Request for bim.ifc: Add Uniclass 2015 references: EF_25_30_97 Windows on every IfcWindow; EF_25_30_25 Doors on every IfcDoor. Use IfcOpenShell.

First a look at what the model holds.

```python
import ifcopenshell

model = ifcopenshell.open("bim.ifc")
print(model.schema)
print("classifications:", [c.Name for c in model.by_type("IfcClassification")])
for ifc_class in ("IfcDoor", "IfcRoof", "IfcStair", "IfcWall", "IfcWindow"):
    print(ifc_class, len(model.by_type(ifc_class)))
```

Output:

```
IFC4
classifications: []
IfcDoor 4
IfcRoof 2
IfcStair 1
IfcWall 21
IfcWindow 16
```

```python
import ifcopenshell
import ifcopenshell.api.classification

model = ifcopenshell.open("bim.ifc")

system = ifcopenshell.api.classification.add_classification(model, classification="Uniclass 2015")

codes = {
    "IfcWindow": ("EF_25_30_97", "Windows"),
    "IfcDoor": ("EF_25_30_25", "Doors"),
}
for ifc_class, (code, name) in codes.items():
    products = model.by_type(ifc_class)
    ifcopenshell.api.classification.add_reference(
        model, products=products, classification=system, identification=code, name=name
    )
    print(code, len(products))

model.write("bim-out.ifc")
```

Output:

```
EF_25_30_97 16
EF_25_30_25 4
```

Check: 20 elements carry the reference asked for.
